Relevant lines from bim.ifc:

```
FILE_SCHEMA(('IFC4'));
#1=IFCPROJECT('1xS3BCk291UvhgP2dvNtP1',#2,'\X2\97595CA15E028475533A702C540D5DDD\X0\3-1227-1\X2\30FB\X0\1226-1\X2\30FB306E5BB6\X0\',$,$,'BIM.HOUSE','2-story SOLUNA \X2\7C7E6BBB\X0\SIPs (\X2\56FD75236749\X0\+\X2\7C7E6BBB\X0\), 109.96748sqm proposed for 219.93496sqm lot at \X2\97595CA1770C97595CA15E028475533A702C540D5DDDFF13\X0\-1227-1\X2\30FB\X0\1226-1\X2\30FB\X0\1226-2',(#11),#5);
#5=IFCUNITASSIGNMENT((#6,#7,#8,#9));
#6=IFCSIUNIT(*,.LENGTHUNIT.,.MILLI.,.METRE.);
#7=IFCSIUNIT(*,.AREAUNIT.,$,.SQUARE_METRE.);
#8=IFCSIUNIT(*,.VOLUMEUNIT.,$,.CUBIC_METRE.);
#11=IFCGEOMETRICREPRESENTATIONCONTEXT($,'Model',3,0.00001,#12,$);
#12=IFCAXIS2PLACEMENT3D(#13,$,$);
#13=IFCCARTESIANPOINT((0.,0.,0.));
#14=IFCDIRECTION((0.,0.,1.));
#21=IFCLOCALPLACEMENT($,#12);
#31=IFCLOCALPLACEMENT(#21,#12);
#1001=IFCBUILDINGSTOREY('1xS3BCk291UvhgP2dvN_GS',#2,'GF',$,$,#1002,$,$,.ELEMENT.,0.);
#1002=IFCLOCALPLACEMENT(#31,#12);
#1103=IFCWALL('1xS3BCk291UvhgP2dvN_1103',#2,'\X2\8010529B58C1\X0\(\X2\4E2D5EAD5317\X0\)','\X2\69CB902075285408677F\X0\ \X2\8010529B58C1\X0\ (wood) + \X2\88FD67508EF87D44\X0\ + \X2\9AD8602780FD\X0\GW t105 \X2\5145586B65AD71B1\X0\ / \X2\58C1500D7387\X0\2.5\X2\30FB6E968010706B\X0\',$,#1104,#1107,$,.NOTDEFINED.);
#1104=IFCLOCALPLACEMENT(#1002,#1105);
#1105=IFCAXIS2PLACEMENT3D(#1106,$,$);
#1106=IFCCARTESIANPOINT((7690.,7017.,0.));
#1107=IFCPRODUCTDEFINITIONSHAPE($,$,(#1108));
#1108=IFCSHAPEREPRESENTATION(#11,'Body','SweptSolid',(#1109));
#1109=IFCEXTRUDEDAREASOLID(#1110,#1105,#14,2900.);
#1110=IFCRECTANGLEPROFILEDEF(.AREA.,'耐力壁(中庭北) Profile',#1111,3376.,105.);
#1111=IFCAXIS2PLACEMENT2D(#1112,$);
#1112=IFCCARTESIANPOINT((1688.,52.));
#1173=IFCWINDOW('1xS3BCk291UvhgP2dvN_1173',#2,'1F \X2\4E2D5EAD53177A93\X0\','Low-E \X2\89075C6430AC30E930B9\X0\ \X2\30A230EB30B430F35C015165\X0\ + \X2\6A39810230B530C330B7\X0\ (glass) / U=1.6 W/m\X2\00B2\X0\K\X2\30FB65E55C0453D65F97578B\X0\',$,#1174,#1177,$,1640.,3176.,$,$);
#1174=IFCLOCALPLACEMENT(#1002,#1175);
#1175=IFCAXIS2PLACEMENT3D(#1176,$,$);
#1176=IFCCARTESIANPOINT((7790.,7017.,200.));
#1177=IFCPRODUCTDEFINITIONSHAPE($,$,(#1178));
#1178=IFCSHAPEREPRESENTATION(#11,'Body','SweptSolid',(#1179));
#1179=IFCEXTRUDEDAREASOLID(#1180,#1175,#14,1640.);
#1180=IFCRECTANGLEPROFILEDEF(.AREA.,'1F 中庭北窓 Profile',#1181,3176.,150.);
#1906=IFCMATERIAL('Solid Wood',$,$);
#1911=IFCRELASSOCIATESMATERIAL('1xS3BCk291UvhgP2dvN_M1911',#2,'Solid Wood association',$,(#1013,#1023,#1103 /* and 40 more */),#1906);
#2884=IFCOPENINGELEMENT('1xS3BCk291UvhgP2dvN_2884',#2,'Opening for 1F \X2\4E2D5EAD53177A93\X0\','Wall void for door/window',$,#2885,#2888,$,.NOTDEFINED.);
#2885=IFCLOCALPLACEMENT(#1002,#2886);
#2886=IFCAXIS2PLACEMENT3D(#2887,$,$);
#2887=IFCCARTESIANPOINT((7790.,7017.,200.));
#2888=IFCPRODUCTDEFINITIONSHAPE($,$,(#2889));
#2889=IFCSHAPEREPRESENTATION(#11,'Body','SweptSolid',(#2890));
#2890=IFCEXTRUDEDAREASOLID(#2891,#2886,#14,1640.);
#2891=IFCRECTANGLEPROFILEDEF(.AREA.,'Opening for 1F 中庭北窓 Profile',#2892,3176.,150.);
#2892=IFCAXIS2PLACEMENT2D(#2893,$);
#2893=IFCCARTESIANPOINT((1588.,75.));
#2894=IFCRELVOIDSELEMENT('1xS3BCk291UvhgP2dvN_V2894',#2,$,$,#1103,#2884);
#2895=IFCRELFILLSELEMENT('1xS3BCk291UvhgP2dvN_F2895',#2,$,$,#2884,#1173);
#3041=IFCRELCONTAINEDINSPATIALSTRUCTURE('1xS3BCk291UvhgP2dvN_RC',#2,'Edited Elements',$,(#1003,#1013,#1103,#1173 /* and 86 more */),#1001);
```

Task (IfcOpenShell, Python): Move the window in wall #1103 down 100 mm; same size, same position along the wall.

```python
import numpy as np
import ifcopenshell
import ifcopenshell.api.geometry
import ifcopenshell.util.placement
import ifcopenshell.util.unit

model = ifcopenshell.open("bim.ifc")
unit_scale = ifcopenshell.util.unit.calculate_unit_scale(model)

window = model.by_guid("1xS3BCk291UvhgP2dvN_1173")
opening = window.FillsVoids[0].RelatingOpeningElement
dz = -0.1 / unit_scale

shift = np.array([0.0, 0.0, dz])
# The window is not placed relative to its opening, so move both.
for product in (opening, window):
    matrix = ifcopenshell.util.placement.get_local_placement(product.ObjectPlacement)
    matrix[:3, 3] += shift
    ifcopenshell.api.geometry.edit_object_placement(model, product=product, matrix=matrix, is_si=False)

print(f"moved by {dz * unit_scale:+.3f} m")

model.write("bim-out.ifc")
```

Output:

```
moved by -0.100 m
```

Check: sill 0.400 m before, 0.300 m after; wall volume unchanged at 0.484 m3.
